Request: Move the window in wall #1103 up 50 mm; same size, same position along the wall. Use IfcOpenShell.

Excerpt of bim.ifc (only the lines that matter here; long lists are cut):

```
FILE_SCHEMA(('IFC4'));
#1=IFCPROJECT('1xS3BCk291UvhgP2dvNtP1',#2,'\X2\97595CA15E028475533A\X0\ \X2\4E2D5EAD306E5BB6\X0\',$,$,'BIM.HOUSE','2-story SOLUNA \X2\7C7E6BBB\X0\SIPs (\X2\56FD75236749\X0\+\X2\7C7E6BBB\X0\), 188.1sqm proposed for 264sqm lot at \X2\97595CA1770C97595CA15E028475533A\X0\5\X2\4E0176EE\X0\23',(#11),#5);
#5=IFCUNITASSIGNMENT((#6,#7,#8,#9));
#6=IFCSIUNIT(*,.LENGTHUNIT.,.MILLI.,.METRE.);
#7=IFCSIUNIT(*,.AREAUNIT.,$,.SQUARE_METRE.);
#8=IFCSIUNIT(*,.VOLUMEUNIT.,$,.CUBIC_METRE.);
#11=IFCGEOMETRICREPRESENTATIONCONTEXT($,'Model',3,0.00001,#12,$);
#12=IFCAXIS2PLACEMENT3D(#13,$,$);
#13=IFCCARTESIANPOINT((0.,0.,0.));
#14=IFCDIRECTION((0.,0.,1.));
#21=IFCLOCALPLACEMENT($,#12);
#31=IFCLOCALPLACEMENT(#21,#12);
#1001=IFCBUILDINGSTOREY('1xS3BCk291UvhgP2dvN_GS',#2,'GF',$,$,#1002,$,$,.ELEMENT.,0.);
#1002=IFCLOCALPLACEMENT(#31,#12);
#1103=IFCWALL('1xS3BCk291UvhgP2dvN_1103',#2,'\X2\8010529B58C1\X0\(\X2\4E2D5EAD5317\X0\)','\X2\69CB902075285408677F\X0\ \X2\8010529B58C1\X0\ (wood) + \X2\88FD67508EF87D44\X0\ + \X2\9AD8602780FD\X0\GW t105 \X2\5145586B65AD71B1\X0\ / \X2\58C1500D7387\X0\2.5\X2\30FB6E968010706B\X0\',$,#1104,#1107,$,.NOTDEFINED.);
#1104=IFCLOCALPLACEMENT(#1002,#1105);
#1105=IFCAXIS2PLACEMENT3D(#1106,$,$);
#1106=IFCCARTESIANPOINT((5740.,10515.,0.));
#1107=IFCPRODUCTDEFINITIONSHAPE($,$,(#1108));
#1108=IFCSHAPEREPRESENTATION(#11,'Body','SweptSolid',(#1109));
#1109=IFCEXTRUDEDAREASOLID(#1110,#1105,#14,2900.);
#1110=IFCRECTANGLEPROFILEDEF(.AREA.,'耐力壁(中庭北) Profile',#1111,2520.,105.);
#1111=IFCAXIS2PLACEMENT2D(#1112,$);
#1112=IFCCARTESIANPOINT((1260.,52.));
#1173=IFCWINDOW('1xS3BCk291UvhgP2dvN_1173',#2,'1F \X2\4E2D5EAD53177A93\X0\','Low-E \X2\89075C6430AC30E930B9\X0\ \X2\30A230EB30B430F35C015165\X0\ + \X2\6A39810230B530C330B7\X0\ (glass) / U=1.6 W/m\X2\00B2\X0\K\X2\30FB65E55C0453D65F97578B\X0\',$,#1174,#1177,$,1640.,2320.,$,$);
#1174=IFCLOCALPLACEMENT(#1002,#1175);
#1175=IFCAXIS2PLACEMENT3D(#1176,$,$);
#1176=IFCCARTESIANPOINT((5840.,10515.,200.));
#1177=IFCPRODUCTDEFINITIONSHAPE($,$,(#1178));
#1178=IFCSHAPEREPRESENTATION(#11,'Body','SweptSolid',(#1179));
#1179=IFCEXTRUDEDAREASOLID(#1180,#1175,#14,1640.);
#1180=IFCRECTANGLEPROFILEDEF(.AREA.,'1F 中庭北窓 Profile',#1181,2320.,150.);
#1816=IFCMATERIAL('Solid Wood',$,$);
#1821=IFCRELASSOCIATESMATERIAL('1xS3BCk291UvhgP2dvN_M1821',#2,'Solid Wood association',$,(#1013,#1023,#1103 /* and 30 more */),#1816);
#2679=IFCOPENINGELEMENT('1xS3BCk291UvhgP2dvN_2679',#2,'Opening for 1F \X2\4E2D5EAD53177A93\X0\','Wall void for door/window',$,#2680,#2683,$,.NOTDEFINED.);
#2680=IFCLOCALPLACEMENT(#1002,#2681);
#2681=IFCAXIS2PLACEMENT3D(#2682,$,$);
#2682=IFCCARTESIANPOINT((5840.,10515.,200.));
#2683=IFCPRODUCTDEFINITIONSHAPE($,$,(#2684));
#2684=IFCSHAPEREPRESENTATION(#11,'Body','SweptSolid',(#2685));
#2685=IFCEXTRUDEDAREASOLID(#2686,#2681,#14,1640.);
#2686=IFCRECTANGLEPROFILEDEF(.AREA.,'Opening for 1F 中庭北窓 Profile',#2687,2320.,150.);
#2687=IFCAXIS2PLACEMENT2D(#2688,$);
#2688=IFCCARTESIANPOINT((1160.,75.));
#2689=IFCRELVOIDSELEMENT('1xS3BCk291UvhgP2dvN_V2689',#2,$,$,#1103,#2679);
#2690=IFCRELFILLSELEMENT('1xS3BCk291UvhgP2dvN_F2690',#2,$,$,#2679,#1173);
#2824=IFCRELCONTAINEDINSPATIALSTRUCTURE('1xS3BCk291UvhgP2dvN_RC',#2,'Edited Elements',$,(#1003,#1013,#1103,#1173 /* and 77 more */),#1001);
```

```python
import numpy as np
import ifcopenshell
import ifcopenshell.api.geometry
import ifcopenshell.util.placement
import ifcopenshell.util.unit

model = ifcopenshell.open("bim.ifc")
unit_scale = ifcopenshell.util.unit.calculate_unit_scale(model)

window = model.by_id(1173)
opening = window.FillsVoids[0].RelatingOpeningElement
dz = 50.0

shift = np.array([0.0, 0.0, dz])
# The window is not placed relative to its opening, so move both.
for product in (opening, window):
    matrix = ifcopenshell.util.placement.get_local_placement(product.ObjectPlacement)
    matrix[:3, 3] += shift
    ifcopenshell.api.geometry.edit_object_placement(model, product=product, matrix=matrix, is_si=False)

print(f"moved by {dz * unit_scale:+.3f} m")

model.write("bim_v2.ifc")
```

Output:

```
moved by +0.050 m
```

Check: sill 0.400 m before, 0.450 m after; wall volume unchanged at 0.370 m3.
